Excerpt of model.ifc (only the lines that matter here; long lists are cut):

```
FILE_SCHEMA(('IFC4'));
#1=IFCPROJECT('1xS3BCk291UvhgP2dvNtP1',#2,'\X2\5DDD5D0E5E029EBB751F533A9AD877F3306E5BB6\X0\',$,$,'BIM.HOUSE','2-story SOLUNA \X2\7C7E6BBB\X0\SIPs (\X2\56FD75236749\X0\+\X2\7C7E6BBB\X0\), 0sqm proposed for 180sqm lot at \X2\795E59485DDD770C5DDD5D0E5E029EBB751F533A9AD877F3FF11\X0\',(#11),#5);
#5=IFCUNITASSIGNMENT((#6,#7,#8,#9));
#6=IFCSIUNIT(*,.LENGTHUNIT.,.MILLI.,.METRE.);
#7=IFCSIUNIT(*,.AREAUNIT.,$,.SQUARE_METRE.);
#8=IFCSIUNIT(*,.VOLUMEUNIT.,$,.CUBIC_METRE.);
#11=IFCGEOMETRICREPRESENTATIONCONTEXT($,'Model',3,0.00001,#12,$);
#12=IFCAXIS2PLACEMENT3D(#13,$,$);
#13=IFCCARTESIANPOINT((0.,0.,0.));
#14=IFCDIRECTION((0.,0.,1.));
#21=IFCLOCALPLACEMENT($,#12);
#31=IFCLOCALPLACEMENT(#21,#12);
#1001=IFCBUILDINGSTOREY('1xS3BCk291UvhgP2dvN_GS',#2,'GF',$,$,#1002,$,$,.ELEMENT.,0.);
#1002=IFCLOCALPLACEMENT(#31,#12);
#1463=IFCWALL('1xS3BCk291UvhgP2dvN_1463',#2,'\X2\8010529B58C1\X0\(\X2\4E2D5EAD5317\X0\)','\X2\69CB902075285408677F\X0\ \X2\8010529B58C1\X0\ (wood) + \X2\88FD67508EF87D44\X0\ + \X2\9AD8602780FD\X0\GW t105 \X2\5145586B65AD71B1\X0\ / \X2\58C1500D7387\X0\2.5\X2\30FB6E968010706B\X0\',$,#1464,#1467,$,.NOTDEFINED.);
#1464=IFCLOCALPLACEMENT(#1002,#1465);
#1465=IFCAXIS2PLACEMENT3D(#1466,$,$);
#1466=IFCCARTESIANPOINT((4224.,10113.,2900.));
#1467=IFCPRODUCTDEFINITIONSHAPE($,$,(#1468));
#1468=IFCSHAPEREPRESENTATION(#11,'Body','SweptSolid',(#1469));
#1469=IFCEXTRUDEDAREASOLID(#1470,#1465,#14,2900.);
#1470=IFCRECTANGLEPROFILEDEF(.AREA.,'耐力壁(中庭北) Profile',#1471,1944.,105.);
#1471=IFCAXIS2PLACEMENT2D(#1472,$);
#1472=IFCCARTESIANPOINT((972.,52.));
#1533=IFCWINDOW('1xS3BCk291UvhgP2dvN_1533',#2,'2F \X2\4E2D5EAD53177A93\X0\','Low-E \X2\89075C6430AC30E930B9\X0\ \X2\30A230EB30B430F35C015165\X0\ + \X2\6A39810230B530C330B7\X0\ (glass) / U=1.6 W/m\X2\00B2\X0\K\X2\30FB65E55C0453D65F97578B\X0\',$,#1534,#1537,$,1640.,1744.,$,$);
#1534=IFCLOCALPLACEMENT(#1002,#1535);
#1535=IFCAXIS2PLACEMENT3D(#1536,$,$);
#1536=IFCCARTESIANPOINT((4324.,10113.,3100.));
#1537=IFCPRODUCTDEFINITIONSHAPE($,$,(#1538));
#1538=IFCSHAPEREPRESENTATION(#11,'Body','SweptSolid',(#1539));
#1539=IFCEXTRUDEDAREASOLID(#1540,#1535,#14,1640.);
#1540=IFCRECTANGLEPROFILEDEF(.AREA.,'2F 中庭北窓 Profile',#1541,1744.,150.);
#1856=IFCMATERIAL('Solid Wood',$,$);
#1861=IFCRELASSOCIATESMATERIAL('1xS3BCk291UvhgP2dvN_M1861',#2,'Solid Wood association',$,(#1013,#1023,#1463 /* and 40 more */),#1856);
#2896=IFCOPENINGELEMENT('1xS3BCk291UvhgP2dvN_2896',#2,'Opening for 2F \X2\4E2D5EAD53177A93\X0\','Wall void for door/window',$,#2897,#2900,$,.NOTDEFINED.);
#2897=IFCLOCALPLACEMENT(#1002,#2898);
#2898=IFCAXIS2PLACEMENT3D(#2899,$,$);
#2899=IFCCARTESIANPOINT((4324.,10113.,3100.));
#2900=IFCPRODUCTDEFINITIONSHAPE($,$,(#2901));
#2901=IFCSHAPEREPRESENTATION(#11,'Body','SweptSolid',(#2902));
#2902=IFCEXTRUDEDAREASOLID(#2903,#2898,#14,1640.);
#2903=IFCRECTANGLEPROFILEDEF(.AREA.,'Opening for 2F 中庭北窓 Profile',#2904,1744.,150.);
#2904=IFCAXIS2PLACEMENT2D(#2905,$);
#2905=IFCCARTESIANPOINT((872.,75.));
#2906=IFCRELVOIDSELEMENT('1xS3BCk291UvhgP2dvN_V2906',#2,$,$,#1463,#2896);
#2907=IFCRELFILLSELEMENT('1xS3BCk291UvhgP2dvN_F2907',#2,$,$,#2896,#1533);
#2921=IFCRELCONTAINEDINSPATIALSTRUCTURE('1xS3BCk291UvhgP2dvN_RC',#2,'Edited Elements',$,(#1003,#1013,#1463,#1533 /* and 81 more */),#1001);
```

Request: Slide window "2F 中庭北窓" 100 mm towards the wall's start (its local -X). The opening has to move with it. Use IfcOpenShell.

```python
import ifcopenshell
import ifcopenshell.api.geometry
import ifcopenshell.util.placement

model = ifcopenshell.open("model.ifc")

window = model.by_guid("1xS3BCk291UvhgP2dvN_1533")
opening = window.FillsVoids[0].RelatingOpeningElement
wall = opening.VoidsElements[0].RelatingBuildingElement

wall_matrix = ifcopenshell.util.placement.get_local_placement(wall.ObjectPlacement)
shift = wall_matrix[:3, 0] * -100.0
before = ifcopenshell.util.placement.get_local_placement(window.ObjectPlacement)[:3, 3].copy()

# The window is not placed relative to its opening, so move both.
for product in (opening, window):
    matrix = ifcopenshell.util.placement.get_local_placement(product.ObjectPlacement)
    matrix[:3, 3] += shift
    ifcopenshell.api.geometry.edit_object_placement(model, product=product, matrix=matrix, is_si=False)

after = ifcopenshell.util.placement.get_local_placement(window.ObjectPlacement)[:3, 3]
print("window moved by", (after - before).round(3) + 0.0)

model.write("model_v2.ifc")
```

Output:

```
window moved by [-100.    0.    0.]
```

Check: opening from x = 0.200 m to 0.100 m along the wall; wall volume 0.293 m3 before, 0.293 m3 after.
